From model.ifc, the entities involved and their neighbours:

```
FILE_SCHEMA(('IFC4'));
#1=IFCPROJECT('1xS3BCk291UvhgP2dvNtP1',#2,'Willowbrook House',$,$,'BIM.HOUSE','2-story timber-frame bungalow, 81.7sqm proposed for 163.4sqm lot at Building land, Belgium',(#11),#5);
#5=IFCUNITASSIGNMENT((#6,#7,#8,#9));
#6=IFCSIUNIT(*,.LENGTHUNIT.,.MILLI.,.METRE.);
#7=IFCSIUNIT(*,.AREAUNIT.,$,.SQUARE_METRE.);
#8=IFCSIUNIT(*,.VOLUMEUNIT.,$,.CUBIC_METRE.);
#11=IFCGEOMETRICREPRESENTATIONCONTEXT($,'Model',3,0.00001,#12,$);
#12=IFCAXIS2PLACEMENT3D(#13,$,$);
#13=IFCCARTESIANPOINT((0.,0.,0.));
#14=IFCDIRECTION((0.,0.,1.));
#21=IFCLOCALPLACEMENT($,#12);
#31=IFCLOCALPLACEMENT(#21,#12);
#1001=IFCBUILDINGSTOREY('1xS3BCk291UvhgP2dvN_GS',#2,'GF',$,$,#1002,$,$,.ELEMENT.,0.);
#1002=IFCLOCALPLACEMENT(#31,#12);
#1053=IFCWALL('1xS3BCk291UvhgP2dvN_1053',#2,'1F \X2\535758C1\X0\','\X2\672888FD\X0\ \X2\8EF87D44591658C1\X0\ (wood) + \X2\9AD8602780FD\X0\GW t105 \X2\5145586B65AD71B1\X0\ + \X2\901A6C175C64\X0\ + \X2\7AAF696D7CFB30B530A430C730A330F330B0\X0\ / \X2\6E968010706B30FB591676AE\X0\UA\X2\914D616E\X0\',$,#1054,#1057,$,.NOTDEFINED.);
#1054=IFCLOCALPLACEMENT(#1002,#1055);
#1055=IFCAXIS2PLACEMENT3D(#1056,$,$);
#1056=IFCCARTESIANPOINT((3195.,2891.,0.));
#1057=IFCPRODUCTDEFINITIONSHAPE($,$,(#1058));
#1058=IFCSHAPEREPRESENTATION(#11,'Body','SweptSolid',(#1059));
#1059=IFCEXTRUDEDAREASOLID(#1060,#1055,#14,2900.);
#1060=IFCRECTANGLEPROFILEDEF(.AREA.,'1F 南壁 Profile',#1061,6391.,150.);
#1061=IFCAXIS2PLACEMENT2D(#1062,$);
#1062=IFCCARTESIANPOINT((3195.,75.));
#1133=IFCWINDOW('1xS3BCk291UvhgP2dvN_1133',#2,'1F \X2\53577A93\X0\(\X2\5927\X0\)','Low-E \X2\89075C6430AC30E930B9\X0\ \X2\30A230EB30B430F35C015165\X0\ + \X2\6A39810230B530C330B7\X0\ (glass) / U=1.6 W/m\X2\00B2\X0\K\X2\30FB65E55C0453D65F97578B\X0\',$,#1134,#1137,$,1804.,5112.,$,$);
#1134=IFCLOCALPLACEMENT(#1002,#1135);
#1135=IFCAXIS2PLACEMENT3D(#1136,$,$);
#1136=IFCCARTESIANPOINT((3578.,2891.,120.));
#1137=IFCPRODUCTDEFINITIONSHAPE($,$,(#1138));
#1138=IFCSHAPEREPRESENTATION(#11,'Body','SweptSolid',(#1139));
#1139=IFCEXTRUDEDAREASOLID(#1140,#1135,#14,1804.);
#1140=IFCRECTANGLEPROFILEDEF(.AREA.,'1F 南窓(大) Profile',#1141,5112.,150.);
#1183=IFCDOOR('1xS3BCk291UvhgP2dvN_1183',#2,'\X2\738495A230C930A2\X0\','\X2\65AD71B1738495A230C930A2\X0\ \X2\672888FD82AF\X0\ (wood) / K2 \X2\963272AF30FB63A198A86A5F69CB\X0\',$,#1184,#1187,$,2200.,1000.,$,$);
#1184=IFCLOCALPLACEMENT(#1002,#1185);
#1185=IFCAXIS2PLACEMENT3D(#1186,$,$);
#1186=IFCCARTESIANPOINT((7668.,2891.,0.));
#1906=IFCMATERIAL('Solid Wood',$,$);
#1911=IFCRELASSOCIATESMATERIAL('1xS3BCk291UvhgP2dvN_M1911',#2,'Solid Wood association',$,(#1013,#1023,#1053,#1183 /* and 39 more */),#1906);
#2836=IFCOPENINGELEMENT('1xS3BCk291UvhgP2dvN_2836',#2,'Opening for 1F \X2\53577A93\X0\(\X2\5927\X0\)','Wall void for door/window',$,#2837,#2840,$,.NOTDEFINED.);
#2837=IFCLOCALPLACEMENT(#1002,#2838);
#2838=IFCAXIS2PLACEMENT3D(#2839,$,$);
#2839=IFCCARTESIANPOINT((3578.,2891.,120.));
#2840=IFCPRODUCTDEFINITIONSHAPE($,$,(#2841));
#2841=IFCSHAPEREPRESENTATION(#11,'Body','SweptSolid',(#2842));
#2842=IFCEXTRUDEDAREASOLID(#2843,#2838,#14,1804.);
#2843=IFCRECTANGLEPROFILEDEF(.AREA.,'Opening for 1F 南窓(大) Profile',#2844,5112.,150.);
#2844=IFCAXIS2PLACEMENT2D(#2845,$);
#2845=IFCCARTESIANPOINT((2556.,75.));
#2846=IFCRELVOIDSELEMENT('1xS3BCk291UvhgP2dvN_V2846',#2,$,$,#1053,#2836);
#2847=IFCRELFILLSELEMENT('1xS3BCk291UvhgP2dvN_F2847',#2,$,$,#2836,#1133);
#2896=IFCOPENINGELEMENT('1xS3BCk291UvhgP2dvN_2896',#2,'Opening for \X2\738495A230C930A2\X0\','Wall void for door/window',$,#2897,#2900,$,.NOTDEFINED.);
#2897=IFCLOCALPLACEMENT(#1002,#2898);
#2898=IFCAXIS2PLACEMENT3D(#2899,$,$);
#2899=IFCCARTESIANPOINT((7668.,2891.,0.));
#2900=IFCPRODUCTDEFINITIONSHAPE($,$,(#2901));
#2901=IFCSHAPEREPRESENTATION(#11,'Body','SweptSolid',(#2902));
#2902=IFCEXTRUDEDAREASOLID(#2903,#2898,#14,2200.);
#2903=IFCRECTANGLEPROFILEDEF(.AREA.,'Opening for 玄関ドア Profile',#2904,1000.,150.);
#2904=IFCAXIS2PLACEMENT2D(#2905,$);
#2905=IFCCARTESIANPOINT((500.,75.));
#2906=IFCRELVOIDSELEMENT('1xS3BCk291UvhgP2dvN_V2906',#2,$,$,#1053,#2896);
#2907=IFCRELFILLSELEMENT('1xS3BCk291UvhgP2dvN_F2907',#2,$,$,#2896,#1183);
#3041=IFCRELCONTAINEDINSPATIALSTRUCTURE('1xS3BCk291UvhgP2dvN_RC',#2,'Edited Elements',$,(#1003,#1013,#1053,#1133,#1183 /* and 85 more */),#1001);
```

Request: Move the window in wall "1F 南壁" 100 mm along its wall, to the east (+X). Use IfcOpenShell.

```python
import ifcopenshell
import ifcopenshell.api.geometry
import ifcopenshell.util.placement
import ifcopenshell.util.unit

model = ifcopenshell.open("model.ifc")
unit_scale = ifcopenshell.util.unit.calculate_unit_scale(model)

window = model.by_guid("1xS3BCk291UvhgP2dvN_1133")
opening = window.FillsVoids[0].RelatingOpeningElement
wall = opening.VoidsElements[0].RelatingBuildingElement

wall_matrix = ifcopenshell.util.placement.get_local_placement(wall.ObjectPlacement)
shift = wall_matrix[:3, 0] * 0.1 / unit_scale
before = ifcopenshell.util.placement.get_local_placement(window.ObjectPlacement)[:3, 3].copy()

# The window is not placed relative to its opening, so move both.
for product in (opening, window):
    matrix = ifcopenshell.util.placement.get_local_placement(product.ObjectPlacement)
    matrix[:3, 3] += shift
    ifcopenshell.api.geometry.edit_object_placement(model, product=product, matrix=matrix, is_si=False)

after = ifcopenshell.util.placement.get_local_placement(window.ObjectPlacement)[:3, 3]
print("window moved by", (after - before).round(3) + 0.0)

model.write("model_updated.ifc")
```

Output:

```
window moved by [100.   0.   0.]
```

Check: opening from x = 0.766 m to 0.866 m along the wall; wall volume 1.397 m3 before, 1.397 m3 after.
